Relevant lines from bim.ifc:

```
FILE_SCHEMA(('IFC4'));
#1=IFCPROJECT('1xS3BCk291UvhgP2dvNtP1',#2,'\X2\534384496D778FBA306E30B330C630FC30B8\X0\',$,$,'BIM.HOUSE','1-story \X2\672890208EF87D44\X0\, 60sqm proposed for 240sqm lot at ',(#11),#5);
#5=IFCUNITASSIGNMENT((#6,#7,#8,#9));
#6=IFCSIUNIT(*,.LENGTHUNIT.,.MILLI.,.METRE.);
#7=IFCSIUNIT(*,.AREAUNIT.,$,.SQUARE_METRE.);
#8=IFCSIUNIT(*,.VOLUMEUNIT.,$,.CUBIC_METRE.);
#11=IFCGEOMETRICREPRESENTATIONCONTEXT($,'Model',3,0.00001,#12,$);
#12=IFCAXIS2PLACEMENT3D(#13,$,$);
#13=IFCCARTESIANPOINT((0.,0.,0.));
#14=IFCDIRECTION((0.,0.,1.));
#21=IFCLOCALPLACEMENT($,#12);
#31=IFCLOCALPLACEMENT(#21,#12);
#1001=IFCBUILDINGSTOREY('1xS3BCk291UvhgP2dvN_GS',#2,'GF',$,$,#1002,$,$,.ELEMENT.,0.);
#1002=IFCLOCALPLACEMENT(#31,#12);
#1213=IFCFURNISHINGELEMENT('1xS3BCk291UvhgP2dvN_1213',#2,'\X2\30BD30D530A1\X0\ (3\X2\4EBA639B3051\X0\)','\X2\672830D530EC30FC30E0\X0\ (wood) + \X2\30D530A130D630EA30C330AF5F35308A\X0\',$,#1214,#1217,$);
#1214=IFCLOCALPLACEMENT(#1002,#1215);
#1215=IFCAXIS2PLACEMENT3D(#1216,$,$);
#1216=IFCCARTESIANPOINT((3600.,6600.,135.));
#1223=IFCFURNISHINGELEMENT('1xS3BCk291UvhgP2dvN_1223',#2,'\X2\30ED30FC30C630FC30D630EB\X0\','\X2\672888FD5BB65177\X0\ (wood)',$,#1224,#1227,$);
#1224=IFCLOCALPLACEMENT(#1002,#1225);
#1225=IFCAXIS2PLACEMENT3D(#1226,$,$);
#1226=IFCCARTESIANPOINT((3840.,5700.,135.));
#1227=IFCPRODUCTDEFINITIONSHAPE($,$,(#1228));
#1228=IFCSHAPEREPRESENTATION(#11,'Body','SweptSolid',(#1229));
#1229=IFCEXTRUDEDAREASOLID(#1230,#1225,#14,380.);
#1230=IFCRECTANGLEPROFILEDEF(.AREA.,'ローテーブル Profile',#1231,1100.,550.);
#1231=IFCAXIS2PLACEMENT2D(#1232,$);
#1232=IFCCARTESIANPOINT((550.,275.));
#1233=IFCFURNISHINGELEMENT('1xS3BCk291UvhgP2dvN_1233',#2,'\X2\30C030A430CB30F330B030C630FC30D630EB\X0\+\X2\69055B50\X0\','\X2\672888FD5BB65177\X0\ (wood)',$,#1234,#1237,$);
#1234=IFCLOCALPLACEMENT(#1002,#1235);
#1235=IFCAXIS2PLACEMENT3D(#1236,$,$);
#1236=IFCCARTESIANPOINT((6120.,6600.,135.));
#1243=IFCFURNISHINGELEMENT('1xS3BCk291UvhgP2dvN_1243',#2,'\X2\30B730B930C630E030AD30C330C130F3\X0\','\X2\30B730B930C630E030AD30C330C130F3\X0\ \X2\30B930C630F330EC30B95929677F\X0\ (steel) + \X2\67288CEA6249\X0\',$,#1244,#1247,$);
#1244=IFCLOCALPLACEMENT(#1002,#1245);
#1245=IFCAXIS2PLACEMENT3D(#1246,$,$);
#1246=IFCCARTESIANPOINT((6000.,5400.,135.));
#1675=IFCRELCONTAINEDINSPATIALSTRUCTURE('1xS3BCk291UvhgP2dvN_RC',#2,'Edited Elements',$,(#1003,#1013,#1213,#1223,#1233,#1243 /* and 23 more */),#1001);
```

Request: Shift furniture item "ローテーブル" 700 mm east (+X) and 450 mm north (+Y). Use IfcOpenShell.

```python
import ifcopenshell
import ifcopenshell.api.geometry
import ifcopenshell.util.placement
import ifcopenshell.util.unit

model = ifcopenshell.open("bim.ifc")
unit_scale = ifcopenshell.util.unit.calculate_unit_scale(model)

item = model.by_guid("1xS3BCk291UvhgP2dvN_1223")
matrix = ifcopenshell.util.placement.get_local_placement(item.ObjectPlacement)
matrix[0, 3] += 0.7 / unit_scale
matrix[1, 3] += 0.45 / unit_scale
ifcopenshell.api.geometry.edit_object_placement(model, product=item, matrix=matrix, is_si=False)

print(ifcopenshell.util.placement.get_local_placement(item.ObjectPlacement).round(3) + 0.0)

model.write("bim_rev.ifc")
```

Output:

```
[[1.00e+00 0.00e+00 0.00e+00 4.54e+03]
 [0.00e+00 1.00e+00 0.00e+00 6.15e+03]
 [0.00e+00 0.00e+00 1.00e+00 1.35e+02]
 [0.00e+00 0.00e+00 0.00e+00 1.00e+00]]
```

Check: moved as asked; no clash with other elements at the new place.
